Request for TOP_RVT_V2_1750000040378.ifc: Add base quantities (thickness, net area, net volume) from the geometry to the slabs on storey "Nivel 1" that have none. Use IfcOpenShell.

First a look at what the model holds.

```python
import ifcopenshell
import ifcopenshell.util.element
import ifcopenshell.util.unit

model = ifcopenshell.open("TOP_RVT_V2_1750000040378.ifc")
print(model.schema)
for unit_type in ("LENGTHUNIT", "AREAUNIT", "VOLUMEUNIT"):
    print(unit_type, ifcopenshell.util.unit.calculate_unit_scale(model, unit_type))
storey = next(s for s in model.by_type("IfcBuildingStorey") if s.Name == "Nivel 1")
slabs = [e for e in ifcopenshell.util.element.get_decomposition(storey) if e.is_a("IfcSlab")]
for e in sorted(slabs, key=lambda e: e.id()):
    print(e.id(), e.is_a(), e.Name, list(ifcopenshell.util.element.get_psets(e, qtos_only=True)), sep=" | ")
```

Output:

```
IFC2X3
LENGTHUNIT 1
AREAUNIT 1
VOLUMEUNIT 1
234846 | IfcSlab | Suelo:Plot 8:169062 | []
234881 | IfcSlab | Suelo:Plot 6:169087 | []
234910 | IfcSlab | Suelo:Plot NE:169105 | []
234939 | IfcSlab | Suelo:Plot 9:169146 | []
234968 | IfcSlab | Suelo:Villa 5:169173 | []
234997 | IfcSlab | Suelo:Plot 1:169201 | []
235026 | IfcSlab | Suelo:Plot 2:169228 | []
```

```python
import ifcopenshell
import ifcopenshell.api.pset
import ifcopenshell.geom
import ifcopenshell.util.element
import ifcopenshell.util.shape
import ifcopenshell.util.unit

model = ifcopenshell.open("TOP_RVT_V2_1750000040378.ifc")
unit_scale = ifcopenshell.util.unit.calculate_unit_scale(model)
area_scale = ifcopenshell.util.unit.calculate_unit_scale(model, "AREAUNIT")
volume_scale = ifcopenshell.util.unit.calculate_unit_scale(model, "VOLUMEUNIT")
settings = ifcopenshell.geom.settings()

storey = next(s for s in model.by_type("IfcBuildingStorey") if s.Name == "Nivel 1")
slabs = [e for e in ifcopenshell.util.element.get_decomposition(storey) if e.is_a("IfcSlab")]

for e in sorted(slabs, key=lambda e: e.id()):
    if ifcopenshell.util.element.get_psets(e, qtos_only=True, should_inherit=False):
        continue
    # Geometry comes back in metres, in the element's own axes.
    shape = ifcopenshell.geom.create_shape(settings, e)
    values = {
        "Width": ifcopenshell.util.shape.get_z(shape.geometry) / unit_scale,
        "NetArea": ifcopenshell.util.shape.get_footprint_area(shape.geometry) / area_scale,
        "NetVolume": ifcopenshell.util.shape.get_volume(shape.geometry) / volume_scale,
    }
    qto = ifcopenshell.api.pset.add_qto(model, product=e, name="BaseQuantities")
    ifcopenshell.api.pset.edit_qto(model, qto=qto, properties=values)
    print(e.id(), {k: round(v, 3) for k, v in values.items()})

model.write("TOP_RVT_V2_1750000040378_updated.ifc")
```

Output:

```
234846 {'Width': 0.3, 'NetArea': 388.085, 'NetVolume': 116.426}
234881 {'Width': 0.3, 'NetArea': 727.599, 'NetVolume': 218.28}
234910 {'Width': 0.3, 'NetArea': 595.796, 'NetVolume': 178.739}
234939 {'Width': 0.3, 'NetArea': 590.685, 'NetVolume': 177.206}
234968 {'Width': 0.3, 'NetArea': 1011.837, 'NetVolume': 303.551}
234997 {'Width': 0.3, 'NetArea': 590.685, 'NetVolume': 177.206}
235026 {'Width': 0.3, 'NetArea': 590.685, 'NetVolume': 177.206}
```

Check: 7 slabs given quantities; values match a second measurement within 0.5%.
